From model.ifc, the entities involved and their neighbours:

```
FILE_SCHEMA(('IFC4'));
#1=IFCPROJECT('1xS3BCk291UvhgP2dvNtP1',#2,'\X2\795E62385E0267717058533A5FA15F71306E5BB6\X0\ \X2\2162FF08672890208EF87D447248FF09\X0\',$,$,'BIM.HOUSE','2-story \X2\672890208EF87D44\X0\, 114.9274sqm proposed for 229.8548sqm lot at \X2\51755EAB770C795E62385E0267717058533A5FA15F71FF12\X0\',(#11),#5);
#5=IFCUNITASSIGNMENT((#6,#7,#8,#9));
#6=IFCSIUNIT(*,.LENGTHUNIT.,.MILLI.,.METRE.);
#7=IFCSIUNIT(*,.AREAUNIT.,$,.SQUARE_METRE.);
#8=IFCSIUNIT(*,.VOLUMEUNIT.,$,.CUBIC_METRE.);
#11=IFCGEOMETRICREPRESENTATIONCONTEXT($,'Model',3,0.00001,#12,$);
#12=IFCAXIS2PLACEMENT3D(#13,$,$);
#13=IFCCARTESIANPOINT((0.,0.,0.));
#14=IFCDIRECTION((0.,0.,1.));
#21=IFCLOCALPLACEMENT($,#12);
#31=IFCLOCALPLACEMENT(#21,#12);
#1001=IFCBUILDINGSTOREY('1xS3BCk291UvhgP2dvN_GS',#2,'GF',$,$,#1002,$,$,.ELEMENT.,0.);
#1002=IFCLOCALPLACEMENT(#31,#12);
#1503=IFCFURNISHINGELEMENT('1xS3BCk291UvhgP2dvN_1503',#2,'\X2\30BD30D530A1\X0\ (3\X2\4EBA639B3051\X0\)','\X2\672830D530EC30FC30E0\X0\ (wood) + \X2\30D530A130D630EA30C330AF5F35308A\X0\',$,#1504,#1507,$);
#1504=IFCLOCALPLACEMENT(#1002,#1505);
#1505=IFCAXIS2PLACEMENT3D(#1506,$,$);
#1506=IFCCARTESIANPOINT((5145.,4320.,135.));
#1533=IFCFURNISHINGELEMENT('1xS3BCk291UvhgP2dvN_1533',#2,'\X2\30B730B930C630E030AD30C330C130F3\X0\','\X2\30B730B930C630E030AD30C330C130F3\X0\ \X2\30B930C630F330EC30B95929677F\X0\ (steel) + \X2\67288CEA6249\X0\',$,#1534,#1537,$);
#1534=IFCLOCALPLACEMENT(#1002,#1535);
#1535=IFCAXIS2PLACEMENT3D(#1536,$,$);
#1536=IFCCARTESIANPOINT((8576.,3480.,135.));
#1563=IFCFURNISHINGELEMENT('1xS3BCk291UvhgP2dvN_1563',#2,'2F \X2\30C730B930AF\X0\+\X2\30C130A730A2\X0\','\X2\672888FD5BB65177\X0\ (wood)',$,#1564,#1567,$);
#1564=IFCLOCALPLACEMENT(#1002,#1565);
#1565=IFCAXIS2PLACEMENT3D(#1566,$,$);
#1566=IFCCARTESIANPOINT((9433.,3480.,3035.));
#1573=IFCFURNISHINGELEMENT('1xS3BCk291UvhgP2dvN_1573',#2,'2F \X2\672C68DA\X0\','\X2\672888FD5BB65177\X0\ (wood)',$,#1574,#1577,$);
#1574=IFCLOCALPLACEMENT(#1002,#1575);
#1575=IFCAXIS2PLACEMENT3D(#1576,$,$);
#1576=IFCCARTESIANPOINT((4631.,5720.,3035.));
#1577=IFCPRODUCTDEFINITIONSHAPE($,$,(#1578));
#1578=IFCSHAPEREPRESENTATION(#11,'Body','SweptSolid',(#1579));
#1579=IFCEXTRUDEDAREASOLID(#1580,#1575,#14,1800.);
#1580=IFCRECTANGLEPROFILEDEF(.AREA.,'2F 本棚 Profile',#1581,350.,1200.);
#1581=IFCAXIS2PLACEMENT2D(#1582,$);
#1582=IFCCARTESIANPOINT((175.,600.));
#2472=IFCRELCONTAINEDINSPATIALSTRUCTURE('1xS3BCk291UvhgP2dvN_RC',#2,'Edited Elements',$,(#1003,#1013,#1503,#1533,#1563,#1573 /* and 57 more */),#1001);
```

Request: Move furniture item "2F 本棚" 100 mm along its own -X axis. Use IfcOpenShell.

```python
import ifcopenshell
import ifcopenshell.api.geometry
import ifcopenshell.util.placement

model = ifcopenshell.open("model.ifc")

item = model.by_guid("1xS3BCk291UvhgP2dvN_1573")
matrix = ifcopenshell.util.placement.get_local_placement(item.ObjectPlacement)
matrix[:3, 3] -= matrix[:3, 0] * 100.0
ifcopenshell.api.geometry.edit_object_placement(model, product=item, matrix=matrix, is_si=False)

print(ifcopenshell.util.placement.get_local_placement(item.ObjectPlacement).round(3) + 0.0)

model.write("model_rev.ifc")
```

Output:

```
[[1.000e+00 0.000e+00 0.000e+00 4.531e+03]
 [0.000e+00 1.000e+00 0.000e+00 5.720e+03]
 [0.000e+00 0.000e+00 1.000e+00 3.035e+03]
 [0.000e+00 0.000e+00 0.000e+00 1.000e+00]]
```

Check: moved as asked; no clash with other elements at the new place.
